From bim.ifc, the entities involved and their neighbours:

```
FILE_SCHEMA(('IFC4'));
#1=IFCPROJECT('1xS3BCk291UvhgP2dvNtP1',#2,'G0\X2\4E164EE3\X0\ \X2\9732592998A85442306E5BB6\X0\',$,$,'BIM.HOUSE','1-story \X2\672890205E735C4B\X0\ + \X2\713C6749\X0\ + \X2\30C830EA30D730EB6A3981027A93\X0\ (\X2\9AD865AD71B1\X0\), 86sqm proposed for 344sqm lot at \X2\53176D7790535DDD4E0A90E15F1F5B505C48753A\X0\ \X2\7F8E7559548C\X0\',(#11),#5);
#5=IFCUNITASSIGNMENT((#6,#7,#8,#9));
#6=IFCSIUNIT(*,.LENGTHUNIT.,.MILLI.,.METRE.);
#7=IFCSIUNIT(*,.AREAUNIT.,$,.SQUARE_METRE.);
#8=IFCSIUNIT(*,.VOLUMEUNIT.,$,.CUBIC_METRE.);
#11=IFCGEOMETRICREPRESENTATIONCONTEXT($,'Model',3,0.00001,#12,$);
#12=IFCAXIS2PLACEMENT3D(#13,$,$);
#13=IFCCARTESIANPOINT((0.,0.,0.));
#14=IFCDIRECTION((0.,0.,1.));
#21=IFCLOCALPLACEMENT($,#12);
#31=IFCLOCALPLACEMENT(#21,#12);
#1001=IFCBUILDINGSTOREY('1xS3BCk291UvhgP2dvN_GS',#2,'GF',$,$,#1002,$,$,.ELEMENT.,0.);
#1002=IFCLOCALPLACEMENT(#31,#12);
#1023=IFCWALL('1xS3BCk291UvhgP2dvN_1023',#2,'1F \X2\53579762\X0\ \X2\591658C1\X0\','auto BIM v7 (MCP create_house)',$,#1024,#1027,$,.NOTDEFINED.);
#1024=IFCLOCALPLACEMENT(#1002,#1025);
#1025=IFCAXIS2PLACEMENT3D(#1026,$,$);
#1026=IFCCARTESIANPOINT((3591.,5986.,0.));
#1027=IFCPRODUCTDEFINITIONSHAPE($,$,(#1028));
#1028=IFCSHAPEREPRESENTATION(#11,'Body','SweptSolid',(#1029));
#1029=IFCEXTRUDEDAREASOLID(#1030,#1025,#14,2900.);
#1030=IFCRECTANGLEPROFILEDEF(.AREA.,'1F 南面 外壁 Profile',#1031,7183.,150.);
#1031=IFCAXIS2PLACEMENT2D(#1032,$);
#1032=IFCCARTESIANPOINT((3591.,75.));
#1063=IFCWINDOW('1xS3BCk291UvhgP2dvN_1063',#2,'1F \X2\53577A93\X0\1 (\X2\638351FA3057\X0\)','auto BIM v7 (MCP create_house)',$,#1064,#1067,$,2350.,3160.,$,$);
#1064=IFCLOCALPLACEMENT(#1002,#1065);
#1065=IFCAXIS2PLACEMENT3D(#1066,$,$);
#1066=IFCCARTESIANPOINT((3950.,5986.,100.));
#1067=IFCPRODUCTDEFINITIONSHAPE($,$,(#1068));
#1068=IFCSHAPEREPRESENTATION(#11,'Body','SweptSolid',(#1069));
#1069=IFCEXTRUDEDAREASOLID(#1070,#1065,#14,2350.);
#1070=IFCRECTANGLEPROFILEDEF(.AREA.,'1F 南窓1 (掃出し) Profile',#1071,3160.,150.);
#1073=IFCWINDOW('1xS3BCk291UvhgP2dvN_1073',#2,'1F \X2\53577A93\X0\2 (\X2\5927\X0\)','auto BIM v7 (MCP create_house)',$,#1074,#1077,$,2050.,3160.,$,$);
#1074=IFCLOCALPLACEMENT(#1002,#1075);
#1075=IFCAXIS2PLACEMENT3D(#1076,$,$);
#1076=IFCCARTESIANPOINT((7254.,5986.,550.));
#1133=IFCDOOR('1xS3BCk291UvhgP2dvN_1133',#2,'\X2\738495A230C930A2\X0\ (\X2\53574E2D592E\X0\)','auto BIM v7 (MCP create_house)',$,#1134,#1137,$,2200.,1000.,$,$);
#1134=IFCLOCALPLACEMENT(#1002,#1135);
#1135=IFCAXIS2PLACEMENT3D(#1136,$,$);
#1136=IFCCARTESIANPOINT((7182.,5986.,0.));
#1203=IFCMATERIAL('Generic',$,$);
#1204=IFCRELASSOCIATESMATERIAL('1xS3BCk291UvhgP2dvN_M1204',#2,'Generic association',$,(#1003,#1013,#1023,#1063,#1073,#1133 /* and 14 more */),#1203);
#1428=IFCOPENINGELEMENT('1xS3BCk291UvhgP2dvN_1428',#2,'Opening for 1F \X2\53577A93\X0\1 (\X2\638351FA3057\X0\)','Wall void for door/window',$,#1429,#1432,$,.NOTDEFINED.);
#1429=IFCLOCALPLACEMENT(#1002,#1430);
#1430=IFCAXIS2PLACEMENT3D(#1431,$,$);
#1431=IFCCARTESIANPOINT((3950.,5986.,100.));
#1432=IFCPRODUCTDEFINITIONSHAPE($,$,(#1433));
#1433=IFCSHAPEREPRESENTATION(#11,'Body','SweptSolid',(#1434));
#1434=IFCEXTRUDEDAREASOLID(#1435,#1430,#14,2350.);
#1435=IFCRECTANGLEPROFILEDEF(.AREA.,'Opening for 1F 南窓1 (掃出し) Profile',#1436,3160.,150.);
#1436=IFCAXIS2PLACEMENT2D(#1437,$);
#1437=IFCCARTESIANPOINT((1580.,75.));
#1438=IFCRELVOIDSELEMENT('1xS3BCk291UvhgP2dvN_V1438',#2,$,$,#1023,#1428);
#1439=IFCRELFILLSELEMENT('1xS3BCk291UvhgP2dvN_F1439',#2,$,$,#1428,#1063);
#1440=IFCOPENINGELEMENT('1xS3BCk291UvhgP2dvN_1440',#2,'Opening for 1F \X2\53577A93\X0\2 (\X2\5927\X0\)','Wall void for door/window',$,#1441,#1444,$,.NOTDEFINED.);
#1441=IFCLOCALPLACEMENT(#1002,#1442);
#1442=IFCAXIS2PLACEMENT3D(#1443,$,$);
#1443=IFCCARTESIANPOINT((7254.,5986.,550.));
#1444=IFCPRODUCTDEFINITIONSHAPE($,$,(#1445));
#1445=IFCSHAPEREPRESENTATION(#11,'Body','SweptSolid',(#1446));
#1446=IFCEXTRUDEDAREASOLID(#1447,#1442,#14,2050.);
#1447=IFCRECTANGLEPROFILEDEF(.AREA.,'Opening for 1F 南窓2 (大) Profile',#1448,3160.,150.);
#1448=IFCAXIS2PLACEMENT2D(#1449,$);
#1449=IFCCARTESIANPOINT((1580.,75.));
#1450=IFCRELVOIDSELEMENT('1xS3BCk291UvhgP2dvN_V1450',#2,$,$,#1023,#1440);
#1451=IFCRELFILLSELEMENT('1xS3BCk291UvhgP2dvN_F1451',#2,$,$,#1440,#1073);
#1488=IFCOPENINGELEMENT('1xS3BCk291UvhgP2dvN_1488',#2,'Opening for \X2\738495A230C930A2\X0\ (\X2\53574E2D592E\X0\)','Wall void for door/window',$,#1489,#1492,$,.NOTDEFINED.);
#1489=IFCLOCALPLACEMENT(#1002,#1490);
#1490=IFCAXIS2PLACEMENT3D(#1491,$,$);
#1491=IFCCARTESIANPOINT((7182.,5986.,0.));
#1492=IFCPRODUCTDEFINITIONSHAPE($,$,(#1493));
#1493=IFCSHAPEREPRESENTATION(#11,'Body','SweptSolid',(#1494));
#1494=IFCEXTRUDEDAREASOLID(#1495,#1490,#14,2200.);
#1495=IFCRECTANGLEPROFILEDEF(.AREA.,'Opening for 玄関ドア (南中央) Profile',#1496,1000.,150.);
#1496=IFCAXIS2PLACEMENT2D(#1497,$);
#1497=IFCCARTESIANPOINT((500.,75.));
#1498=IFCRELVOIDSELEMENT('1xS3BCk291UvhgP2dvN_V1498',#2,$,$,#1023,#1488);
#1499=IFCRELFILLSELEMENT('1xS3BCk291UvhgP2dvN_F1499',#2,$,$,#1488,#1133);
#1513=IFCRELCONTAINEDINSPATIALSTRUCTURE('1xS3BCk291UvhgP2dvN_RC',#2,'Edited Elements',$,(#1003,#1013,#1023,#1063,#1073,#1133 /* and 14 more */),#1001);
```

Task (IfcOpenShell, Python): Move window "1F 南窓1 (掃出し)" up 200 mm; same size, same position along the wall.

```python
import numpy as np
import ifcopenshell
import ifcopenshell.api.geometry
import ifcopenshell.util.placement
import ifcopenshell.util.unit

model = ifcopenshell.open("bim.ifc")
unit_scale = ifcopenshell.util.unit.calculate_unit_scale(model)

window = model.by_guid("1xS3BCk291UvhgP2dvN_1063")
opening = window.FillsVoids[0].RelatingOpeningElement
dz = 0.2 / unit_scale

shift = np.array([0.0, 0.0, dz])
# The window is not placed relative to its opening, so move both.
for product in (opening, window):
    matrix = ifcopenshell.util.placement.get_local_placement(product.ObjectPlacement)
    matrix[:3, 3] += shift
    ifcopenshell.api.geometry.edit_object_placement(model, product=product, matrix=matrix, is_si=False)

print(f"moved by {dz * unit_scale:+.3f} m")

model.write("bim_edited.ifc")
```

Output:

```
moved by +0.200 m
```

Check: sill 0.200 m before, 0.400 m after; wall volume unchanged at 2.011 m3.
